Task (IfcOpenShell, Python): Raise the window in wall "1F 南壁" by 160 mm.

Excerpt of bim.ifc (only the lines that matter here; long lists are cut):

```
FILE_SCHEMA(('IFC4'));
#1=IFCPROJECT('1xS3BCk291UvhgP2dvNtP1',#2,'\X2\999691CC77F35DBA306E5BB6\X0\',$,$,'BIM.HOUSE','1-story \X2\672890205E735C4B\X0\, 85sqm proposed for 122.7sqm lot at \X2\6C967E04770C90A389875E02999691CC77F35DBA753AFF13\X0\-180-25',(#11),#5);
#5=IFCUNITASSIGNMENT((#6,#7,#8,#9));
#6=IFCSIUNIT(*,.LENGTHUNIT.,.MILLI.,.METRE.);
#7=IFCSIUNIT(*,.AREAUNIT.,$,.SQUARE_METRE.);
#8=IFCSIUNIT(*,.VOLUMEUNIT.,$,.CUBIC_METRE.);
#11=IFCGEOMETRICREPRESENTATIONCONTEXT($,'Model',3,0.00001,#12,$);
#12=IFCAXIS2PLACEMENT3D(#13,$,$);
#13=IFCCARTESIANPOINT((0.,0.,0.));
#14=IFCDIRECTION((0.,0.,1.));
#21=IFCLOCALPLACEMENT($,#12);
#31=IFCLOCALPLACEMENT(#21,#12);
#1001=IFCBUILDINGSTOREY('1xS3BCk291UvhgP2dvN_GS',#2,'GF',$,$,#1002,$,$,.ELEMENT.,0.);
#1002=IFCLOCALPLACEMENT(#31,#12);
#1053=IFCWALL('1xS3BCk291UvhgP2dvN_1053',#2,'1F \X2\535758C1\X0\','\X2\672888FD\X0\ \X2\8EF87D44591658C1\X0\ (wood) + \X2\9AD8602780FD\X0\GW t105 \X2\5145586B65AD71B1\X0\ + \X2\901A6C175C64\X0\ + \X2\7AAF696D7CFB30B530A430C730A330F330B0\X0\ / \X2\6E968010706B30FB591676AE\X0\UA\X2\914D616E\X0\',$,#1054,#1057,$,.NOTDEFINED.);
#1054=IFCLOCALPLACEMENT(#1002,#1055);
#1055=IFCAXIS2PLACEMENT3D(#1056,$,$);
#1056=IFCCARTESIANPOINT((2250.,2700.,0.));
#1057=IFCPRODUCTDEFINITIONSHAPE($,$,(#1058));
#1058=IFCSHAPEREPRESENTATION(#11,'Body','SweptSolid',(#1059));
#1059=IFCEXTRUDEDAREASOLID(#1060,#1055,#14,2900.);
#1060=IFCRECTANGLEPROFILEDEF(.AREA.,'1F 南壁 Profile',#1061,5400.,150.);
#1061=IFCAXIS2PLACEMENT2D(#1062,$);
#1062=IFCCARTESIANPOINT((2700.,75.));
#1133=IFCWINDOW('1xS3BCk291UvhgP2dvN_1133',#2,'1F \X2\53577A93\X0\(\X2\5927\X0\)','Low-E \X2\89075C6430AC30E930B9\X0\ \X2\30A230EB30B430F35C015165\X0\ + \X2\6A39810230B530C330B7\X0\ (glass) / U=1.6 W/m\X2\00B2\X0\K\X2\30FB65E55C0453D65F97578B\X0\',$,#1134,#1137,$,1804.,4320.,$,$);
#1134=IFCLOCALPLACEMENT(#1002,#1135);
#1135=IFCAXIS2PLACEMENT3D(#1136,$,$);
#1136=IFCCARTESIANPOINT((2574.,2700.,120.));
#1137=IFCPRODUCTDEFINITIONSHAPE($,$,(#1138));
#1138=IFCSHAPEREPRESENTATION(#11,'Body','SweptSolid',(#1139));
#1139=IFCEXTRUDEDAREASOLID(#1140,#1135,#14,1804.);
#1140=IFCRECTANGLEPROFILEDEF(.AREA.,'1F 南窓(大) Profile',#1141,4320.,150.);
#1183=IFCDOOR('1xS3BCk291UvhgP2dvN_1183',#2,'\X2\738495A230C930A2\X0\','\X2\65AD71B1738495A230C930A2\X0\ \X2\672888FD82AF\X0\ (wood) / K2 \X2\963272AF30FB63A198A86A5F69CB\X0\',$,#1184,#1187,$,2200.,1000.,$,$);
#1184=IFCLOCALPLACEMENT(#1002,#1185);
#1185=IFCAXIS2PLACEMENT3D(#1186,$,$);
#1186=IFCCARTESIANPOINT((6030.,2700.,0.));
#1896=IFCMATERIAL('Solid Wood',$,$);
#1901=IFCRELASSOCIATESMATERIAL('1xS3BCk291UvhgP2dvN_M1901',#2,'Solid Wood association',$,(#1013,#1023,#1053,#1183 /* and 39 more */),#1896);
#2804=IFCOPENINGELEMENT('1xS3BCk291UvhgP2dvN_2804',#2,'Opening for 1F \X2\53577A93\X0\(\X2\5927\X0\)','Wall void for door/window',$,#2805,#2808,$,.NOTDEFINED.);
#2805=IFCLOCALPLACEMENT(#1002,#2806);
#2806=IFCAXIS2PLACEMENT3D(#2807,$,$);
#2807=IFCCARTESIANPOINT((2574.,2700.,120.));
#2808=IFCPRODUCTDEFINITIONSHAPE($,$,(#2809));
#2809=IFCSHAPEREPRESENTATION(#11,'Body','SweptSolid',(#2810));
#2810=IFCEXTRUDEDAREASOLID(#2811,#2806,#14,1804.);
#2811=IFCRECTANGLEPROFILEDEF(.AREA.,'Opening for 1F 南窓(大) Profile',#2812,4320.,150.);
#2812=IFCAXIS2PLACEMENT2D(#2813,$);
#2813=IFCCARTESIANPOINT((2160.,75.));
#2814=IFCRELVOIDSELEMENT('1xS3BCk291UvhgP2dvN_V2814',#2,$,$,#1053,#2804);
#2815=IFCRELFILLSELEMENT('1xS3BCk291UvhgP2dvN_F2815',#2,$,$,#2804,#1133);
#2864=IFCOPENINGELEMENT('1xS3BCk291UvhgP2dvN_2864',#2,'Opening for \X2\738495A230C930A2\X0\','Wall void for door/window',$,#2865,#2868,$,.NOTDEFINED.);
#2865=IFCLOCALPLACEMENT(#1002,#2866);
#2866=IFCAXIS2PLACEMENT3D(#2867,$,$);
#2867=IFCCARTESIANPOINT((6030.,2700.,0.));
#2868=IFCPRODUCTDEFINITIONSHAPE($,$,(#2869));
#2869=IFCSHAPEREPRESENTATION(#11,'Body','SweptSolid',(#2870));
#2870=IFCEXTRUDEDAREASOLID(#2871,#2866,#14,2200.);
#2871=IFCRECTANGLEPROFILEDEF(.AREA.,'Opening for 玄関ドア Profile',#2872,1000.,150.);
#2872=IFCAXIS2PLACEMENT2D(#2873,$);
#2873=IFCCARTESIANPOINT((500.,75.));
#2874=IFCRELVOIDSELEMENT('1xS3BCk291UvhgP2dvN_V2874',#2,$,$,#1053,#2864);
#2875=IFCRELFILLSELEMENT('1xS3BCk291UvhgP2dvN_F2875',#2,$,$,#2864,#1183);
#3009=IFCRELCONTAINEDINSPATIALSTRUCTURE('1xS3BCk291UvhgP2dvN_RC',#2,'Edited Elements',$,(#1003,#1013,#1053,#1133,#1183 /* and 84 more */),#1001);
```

```python
import numpy as np
import ifcopenshell
import ifcopenshell.api.geometry
import ifcopenshell.util.placement
import ifcopenshell.util.unit

model = ifcopenshell.open("bim.ifc")
unit_scale = ifcopenshell.util.unit.calculate_unit_scale(model)

window = model.by_guid("1xS3BCk291UvhgP2dvN_1133")
opening = window.FillsVoids[0].RelatingOpeningElement
dz = 160.0

shift = np.array([0.0, 0.0, dz])
# The window is not placed relative to its opening, so move both.
for product in (opening, window):
    matrix = ifcopenshell.util.placement.get_local_placement(product.ObjectPlacement)
    matrix[:3, 3] += shift
    ifcopenshell.api.geometry.edit_object_placement(model, product=product, matrix=matrix, is_si=False)

print(f"moved by {dz * unit_scale:+.3f} m")

model.write("bim_rev.ifc")
```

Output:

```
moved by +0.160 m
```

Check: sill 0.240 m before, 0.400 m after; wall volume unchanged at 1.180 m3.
